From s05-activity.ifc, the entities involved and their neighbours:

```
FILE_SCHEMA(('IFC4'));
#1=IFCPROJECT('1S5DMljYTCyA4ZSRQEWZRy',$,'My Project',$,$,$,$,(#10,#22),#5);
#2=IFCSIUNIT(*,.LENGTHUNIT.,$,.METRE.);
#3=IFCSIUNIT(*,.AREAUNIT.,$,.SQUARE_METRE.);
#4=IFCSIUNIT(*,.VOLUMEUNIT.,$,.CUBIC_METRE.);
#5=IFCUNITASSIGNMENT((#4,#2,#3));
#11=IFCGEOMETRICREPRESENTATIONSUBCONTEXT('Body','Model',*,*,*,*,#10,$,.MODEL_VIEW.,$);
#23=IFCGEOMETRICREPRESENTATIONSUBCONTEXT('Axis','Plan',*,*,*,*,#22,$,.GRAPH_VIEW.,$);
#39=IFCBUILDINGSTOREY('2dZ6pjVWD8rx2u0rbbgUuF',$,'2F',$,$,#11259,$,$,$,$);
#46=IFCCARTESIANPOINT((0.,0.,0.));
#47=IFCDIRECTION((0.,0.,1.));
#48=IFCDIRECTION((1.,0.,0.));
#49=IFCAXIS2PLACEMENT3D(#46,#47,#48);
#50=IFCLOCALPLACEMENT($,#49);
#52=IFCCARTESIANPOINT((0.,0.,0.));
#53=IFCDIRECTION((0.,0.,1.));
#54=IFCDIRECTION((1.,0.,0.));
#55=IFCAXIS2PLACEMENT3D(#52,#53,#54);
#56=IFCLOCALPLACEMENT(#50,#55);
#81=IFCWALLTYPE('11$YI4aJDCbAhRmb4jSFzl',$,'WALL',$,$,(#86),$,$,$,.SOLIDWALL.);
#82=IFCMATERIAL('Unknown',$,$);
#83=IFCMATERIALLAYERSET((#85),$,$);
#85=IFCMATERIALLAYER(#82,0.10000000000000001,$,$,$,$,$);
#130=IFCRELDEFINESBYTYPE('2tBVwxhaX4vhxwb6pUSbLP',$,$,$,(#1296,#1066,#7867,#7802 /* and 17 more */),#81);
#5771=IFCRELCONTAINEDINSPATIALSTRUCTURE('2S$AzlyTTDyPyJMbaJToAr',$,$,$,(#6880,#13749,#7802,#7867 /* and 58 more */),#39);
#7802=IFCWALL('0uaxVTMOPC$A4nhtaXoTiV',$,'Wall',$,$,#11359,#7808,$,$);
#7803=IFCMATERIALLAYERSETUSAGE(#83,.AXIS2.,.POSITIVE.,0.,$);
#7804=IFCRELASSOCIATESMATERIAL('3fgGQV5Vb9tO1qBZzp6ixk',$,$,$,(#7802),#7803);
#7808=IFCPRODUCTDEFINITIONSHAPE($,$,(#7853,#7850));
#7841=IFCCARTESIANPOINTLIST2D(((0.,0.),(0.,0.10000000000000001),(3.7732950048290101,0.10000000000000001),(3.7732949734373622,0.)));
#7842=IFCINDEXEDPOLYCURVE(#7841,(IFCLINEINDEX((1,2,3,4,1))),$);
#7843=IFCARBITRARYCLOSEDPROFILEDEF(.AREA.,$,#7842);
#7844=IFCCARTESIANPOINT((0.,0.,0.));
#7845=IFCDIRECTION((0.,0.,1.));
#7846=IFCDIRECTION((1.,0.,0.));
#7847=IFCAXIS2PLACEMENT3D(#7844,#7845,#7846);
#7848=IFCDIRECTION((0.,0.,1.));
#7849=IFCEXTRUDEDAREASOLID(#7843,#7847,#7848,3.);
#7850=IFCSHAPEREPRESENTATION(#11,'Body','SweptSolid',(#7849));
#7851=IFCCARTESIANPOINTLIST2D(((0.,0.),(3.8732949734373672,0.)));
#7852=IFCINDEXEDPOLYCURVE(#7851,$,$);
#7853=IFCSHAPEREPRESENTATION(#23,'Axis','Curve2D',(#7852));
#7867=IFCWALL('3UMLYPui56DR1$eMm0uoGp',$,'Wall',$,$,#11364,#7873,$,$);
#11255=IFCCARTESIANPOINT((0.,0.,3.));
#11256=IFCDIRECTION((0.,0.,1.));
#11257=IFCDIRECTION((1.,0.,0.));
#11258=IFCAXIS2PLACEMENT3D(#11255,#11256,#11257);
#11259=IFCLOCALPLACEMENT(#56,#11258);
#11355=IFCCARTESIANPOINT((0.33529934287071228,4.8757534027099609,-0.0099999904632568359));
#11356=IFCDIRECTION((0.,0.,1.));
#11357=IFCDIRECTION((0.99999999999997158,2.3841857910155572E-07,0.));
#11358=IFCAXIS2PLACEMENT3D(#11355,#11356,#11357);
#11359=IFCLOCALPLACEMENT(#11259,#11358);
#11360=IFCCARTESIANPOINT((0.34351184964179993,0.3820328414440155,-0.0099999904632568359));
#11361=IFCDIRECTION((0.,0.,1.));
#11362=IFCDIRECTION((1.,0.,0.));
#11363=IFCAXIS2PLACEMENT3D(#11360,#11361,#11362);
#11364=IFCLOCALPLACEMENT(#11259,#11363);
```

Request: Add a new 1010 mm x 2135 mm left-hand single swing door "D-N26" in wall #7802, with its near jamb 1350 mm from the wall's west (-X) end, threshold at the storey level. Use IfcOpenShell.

```python
import numpy as np
import ifcopenshell
import ifcopenshell.api.feature
import ifcopenshell.api.geometry
import ifcopenshell.api.root
import ifcopenshell.api.spatial
import ifcopenshell.geom
import ifcopenshell.util.element
import ifcopenshell.util.placement
import ifcopenshell.util.representation
import ifcopenshell.util.shape
import ifcopenshell.util.unit

model = ifcopenshell.open("s05-activity.ifc")
unit_scale = ifcopenshell.util.unit.calculate_unit_scale(model)
settings = ifcopenshell.geom.settings()


def volume(element):
    """Net volume in cubic metres, openings subtracted."""
    shape = ifcopenshell.geom.create_shape(settings, element)
    return ifcopenshell.util.shape.get_volume(shape.geometry)


wall = model.by_id(7802)
storey = ifcopenshell.util.element.get_container(wall, ifc_class="IfcBuildingStorey")
context = ifcopenshell.util.representation.get_context(model, "Model", "Body", "MODEL_VIEW")
before = volume(wall)

width, height, from_end, sill = 1.01, 2.135, 1.35, 0.0  # metres

# The wall runs along its own X axis, and the end named is its -X end.
wall_shape = ifcopenshell.geom.create_shape(settings, wall)
x, y, z = ifcopenshell.util.shape.get_vertices(wall_shape.geometry).T
start = x.min() + from_end
face, thickness = float(y.min()), float(y.max() - y.min())
wall_matrix = ifcopenshell.util.placement.get_local_placement(wall.ObjectPlacement)
level = ifcopenshell.util.placement.get_local_placement(storey.ObjectPlacement)[2, 3]


def in_wall(x, y):
    """Placement at x, y metres in the wall's axes, at sill height."""
    matrix = wall_matrix.copy()
    matrix[:, 3] = wall_matrix @ np.array([x / unit_scale, y / unit_scale, 0.0, 1.0])
    matrix[2, 3] = level + sill / unit_scale
    return matrix


# Opening: a box that overshoots both wall faces by 50 mm.
opening = ifcopenshell.api.root.create_entity(model, ifc_class="IfcOpeningElement", predefined_type="OPENING")
box = ifcopenshell.api.geometry.add_wall_representation(
    model, context=context, length=width, height=height, thickness=thickness + 0.1
)
ifcopenshell.api.geometry.assign_representation(model, product=opening, representation=box)
ifcopenshell.api.geometry.edit_object_placement(model, product=opening, matrix=in_wall(start, face - 0.05), is_si=False)
ifcopenshell.api.feature.add_feature(model, feature=opening, element=wall)

door = ifcopenshell.api.root.create_entity(model, ifc_class="IfcDoor", name="D-N26", predefined_type="DOOR")
door.OverallWidth, door.OverallHeight = width / unit_scale, height / unit_scale
door.OperationType = "SINGLE_SWING_LEFT"
body = ifcopenshell.api.geometry.add_door_representation(
    model,
    context=context,
    overall_width=door.OverallWidth,
    overall_height=door.OverallHeight,
    operation_type="SINGLE_SWING_LEFT",
    lining_properties={"LiningDepth": thickness / unit_scale, "ThresholdDepth": thickness / unit_scale},
)
ifcopenshell.api.geometry.assign_representation(model, product=door, representation=body)
ifcopenshell.api.spatial.assign_container(model, products=[door], relating_structure=storey)
ifcopenshell.api.feature.add_filling(model, opening=opening, element=door)

# The lining spans the wall, so the door starts at the wall face.
ifcopenshell.api.geometry.edit_object_placement(model, product=door, matrix=in_wall(start, face), is_si=False)

after = volume(wall)

print(f"wall volume {before:.3f} -> {after:.3f} m3")

model.write("s05-activity_edited.ifc")
```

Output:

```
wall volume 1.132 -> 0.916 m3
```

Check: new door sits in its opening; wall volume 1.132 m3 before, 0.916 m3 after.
